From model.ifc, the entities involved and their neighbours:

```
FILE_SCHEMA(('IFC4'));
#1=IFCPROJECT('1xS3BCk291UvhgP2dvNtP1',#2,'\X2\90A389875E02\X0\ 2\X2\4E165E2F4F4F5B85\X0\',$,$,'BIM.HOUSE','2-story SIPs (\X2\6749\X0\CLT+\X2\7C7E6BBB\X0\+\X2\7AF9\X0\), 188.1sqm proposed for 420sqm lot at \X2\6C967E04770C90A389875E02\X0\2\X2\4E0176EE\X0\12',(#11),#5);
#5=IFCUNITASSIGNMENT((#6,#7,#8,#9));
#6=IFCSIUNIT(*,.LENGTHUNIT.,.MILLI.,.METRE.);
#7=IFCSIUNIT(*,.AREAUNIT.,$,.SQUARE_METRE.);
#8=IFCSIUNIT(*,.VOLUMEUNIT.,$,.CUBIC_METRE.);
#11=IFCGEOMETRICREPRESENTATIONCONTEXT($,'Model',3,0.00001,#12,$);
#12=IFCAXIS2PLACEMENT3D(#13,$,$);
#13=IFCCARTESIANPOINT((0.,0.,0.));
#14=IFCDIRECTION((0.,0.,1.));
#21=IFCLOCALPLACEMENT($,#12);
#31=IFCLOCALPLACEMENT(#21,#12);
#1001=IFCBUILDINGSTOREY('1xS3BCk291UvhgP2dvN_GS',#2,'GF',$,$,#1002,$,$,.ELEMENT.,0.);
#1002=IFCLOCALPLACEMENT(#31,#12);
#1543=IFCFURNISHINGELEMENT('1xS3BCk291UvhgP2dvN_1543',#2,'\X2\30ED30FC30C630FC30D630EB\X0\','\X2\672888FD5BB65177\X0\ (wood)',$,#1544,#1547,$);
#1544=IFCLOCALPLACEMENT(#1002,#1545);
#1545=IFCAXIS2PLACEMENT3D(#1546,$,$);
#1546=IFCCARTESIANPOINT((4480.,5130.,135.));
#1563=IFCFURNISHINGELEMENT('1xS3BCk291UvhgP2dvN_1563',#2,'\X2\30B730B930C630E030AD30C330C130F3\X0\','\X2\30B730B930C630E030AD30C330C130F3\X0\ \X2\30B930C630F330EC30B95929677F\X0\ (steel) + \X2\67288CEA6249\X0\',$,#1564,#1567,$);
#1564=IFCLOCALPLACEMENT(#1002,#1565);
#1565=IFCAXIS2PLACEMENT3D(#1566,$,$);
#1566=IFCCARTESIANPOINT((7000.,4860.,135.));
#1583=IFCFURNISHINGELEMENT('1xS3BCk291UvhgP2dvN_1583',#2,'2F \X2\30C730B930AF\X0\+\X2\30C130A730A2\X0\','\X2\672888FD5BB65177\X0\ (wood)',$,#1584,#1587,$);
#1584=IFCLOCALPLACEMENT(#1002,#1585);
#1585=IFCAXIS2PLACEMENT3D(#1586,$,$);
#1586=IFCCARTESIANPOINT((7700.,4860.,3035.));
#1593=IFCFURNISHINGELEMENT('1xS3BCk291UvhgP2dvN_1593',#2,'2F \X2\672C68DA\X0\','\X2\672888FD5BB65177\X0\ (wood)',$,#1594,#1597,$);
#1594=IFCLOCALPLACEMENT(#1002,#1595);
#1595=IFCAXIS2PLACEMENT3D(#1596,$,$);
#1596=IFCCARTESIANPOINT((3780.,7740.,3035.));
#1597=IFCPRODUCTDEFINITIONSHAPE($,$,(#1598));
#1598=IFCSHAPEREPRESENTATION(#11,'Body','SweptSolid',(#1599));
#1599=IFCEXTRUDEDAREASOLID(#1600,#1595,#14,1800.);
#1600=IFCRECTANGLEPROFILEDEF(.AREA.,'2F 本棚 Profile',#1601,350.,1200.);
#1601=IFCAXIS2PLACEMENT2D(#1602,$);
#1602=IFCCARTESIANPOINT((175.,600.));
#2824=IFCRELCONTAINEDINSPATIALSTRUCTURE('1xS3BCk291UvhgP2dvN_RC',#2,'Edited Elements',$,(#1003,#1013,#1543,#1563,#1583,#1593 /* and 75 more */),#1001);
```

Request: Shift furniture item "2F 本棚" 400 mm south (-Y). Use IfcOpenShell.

```python
import ifcopenshell
import ifcopenshell.api.geometry
import ifcopenshell.util.placement
import ifcopenshell.util.unit

model = ifcopenshell.open("model.ifc")
unit_scale = ifcopenshell.util.unit.calculate_unit_scale(model)

item = model.by_id(1593)
matrix = ifcopenshell.util.placement.get_local_placement(item.ObjectPlacement)
matrix[1, 3] -= 0.4 / unit_scale
ifcopenshell.api.geometry.edit_object_placement(model, product=item, matrix=matrix, is_si=False)

print(ifcopenshell.util.placement.get_local_placement(item.ObjectPlacement).round(3) + 0.0)

model.write("model_rev.ifc")
```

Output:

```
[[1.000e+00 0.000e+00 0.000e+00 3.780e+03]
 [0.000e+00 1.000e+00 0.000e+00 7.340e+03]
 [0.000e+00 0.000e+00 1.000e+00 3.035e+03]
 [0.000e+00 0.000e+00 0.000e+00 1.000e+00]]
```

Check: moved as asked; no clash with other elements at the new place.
